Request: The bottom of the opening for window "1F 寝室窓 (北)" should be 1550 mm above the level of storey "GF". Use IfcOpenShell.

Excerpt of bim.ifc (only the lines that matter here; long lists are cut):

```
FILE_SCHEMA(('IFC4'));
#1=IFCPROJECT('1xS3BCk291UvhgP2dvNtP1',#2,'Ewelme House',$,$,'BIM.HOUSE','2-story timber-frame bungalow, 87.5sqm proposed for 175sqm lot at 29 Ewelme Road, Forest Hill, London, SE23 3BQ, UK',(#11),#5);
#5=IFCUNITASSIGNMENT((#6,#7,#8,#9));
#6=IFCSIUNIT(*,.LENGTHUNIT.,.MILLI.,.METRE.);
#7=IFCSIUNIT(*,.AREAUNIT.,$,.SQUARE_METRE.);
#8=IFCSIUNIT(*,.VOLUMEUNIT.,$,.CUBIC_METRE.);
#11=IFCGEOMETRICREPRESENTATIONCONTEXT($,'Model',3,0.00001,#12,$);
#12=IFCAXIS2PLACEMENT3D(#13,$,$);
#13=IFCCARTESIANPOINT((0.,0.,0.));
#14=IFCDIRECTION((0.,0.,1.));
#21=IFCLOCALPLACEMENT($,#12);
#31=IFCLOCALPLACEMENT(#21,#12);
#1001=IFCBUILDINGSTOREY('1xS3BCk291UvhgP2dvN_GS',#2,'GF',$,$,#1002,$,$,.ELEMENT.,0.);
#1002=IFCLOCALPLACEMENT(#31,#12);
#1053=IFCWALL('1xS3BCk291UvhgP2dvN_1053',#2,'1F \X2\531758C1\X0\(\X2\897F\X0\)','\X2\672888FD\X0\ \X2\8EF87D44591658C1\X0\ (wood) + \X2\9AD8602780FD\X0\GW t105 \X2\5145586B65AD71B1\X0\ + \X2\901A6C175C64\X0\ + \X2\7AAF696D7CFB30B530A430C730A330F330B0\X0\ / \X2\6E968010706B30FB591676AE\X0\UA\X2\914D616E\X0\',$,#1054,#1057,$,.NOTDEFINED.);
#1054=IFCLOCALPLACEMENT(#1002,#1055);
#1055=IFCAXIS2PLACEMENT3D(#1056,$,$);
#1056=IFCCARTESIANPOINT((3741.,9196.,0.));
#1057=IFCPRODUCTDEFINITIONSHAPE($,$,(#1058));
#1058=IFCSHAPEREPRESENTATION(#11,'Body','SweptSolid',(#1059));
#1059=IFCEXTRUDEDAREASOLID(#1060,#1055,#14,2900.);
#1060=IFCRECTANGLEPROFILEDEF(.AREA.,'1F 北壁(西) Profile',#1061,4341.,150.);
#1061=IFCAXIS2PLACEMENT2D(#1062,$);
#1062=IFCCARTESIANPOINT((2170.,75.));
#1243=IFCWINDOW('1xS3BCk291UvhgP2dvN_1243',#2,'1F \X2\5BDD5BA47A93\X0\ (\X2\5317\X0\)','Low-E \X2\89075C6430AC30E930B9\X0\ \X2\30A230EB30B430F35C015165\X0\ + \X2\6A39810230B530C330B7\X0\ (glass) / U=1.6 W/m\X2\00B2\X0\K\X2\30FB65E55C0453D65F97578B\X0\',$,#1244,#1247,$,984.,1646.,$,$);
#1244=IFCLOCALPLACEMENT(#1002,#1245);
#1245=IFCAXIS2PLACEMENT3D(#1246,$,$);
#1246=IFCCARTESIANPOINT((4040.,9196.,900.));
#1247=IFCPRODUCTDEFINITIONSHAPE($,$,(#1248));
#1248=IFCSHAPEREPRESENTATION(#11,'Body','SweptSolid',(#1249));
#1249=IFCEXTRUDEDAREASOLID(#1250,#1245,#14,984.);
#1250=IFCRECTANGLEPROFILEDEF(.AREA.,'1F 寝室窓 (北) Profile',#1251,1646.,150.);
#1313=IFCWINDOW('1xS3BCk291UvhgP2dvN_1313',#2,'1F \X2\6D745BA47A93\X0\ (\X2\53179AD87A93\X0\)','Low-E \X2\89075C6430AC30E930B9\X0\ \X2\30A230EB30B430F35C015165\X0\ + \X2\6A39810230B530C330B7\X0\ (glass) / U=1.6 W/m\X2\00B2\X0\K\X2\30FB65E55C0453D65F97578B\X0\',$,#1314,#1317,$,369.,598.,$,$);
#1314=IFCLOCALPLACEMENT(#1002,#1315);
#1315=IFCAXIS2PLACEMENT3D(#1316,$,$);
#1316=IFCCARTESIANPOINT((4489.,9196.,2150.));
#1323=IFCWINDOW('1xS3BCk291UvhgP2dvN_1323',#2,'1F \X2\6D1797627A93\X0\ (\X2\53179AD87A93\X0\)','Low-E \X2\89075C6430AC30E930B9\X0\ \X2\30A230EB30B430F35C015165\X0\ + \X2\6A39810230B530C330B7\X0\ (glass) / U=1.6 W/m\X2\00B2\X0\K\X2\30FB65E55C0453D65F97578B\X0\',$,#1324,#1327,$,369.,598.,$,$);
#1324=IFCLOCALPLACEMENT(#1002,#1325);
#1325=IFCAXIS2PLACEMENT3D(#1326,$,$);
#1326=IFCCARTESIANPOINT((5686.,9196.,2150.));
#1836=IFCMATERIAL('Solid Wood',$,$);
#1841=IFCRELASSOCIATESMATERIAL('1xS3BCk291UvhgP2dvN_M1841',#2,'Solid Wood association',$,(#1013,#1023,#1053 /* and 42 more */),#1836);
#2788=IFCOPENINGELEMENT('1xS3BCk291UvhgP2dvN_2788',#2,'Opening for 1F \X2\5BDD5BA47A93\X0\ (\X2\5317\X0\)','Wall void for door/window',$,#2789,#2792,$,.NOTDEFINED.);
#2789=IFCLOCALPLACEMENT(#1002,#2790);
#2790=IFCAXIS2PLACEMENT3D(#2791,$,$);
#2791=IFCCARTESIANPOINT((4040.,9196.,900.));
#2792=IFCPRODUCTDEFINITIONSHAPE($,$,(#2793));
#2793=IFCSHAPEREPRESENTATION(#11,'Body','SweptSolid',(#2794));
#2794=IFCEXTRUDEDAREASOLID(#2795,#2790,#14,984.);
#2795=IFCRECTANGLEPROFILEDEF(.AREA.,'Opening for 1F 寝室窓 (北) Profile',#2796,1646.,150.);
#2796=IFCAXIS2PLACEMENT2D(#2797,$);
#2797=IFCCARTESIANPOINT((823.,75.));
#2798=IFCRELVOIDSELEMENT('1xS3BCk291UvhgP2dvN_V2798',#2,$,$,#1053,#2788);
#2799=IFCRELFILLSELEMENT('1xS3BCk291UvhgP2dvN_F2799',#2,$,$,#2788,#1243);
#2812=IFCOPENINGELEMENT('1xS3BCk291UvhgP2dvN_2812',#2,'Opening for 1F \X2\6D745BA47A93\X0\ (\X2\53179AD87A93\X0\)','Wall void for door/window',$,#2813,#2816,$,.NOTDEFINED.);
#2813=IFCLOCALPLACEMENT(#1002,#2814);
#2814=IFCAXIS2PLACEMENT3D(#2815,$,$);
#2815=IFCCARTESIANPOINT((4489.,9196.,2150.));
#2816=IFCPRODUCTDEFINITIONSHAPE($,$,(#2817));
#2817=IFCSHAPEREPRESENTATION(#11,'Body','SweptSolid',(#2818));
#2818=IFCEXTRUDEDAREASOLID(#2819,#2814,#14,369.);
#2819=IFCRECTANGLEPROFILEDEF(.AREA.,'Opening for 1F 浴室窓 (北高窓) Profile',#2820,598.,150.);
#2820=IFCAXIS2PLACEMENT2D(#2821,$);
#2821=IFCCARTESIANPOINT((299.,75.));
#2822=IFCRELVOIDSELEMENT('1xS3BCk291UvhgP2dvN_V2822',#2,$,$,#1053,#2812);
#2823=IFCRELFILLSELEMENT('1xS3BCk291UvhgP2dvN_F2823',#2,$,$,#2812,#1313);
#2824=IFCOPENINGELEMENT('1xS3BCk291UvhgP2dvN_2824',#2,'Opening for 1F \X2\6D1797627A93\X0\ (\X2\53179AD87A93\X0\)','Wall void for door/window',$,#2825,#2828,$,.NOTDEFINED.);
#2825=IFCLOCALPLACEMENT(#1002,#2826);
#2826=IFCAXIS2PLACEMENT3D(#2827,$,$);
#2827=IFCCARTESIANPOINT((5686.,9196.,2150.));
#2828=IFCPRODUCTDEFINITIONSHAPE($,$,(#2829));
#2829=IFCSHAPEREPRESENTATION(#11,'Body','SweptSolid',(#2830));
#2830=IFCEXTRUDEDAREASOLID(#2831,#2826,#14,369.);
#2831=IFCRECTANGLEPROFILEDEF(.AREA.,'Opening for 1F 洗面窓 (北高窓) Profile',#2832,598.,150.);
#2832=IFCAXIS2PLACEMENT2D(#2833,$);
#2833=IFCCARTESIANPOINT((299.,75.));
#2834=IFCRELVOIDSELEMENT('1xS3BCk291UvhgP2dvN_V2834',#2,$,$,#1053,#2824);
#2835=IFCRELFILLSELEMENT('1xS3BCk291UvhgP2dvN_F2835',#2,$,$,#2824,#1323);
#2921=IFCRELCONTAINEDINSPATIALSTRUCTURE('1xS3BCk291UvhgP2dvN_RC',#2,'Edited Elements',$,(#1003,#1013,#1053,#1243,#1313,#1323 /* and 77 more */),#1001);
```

```python
import numpy as np
import ifcopenshell
import ifcopenshell.api.geometry
import ifcopenshell.geom
import ifcopenshell.util.element
import ifcopenshell.util.placement
import ifcopenshell.util.shape
import ifcopenshell.util.unit

model = ifcopenshell.open("bim.ifc")
unit_scale = ifcopenshell.util.unit.calculate_unit_scale(model)

window = model.by_guid("1xS3BCk291UvhgP2dvN_1243")
opening = window.FillsVoids[0].RelatingOpeningElement
storey = ifcopenshell.util.element.get_container(window, ifc_class="IfcBuildingStorey")
level = ifcopenshell.util.placement.get_local_placement(storey.ObjectPlacement)[2, 3]

# The opening's origin need not be at the sill, so measure its lowest point.
shape = ifcopenshell.geom.create_shape(ifcopenshell.geom.settings(), opening)
bottom = ifcopenshell.util.shape.get_shape_bottom_elevation(shape, shape.geometry) / unit_scale
dz = level + 1.55 / unit_scale - bottom

shift = np.array([0.0, 0.0, dz])
# The window is not placed relative to its opening, so move both.
for product in (opening, window):
    matrix = ifcopenshell.util.placement.get_local_placement(product.ObjectPlacement)
    matrix[:3, 3] += shift
    ifcopenshell.api.geometry.edit_object_placement(model, product=product, matrix=matrix, is_si=False)

print(f"moved by {dz * unit_scale:+.3f} m")

model.write("bim_updated.ifc")
```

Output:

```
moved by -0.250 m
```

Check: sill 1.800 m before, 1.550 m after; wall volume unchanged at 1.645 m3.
